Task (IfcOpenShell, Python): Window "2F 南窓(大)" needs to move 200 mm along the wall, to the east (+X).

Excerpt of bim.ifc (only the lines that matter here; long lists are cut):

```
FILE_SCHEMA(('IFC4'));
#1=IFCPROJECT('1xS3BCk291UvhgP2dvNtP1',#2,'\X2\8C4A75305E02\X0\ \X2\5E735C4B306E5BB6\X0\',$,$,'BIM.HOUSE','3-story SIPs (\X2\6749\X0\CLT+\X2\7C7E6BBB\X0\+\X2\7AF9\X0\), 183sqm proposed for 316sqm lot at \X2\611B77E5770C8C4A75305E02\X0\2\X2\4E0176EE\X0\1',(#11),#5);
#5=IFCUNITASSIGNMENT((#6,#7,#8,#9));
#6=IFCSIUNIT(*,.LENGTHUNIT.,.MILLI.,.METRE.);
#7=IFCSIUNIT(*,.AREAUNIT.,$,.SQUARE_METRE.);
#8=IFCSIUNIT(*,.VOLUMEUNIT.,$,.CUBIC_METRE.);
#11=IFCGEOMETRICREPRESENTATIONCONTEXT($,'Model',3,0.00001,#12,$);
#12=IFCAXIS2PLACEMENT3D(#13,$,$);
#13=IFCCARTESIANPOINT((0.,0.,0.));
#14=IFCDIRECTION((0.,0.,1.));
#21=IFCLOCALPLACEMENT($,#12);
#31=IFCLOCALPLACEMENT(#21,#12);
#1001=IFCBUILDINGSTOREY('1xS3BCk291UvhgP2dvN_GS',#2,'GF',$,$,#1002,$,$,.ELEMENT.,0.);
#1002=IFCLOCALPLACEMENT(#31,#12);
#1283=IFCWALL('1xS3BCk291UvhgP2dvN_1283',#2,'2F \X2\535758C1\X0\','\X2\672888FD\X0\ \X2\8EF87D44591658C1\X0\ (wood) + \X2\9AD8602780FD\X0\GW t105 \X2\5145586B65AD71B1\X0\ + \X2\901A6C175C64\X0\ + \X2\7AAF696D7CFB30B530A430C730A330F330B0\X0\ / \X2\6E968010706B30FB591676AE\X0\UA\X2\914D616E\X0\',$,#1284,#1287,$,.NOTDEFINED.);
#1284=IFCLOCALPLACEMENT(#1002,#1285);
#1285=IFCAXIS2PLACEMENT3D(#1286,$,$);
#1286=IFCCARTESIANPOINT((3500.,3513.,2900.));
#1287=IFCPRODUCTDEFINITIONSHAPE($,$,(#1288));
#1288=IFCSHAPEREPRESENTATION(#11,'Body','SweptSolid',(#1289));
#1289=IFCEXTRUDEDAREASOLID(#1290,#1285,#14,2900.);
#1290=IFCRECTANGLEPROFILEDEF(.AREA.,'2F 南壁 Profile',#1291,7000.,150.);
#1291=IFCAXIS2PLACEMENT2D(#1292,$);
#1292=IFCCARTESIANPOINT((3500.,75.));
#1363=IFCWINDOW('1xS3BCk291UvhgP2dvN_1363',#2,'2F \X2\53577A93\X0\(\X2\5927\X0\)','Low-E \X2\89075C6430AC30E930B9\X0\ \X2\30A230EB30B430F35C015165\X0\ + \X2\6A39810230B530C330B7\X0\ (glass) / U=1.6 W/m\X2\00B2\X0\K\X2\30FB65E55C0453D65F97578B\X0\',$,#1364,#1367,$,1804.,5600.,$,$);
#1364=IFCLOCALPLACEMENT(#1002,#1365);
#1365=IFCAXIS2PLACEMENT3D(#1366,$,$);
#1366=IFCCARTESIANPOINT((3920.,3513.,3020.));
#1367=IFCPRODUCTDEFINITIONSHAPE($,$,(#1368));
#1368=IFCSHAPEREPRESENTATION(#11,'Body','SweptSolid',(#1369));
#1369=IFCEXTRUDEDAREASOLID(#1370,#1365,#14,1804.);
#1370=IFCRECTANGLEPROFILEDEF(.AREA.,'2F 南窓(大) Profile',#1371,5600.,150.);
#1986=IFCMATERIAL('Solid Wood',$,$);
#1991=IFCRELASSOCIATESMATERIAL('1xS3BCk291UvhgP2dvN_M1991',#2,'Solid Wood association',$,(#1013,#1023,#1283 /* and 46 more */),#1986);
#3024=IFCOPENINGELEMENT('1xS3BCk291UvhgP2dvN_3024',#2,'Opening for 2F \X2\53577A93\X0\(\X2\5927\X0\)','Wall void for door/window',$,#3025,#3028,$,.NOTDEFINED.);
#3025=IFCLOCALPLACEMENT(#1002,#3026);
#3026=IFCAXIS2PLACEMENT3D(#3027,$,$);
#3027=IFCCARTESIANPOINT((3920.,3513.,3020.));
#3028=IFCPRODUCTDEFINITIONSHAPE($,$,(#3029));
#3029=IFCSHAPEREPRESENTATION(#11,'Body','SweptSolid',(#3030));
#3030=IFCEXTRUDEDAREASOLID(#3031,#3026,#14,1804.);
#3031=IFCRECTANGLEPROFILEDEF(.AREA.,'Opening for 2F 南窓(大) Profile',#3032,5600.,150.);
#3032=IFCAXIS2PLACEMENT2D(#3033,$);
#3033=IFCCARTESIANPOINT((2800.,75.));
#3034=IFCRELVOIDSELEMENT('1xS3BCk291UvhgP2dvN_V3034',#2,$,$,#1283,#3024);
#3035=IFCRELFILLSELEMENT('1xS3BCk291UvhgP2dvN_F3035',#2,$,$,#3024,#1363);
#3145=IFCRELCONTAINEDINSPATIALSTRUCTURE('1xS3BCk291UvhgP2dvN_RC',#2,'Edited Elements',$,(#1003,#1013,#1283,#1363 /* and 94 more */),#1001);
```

```python
import ifcopenshell
import ifcopenshell.api.geometry
import ifcopenshell.util.placement
import ifcopenshell.util.unit

model = ifcopenshell.open("bim.ifc")
unit_scale = ifcopenshell.util.unit.calculate_unit_scale(model)

window = model.by_guid("1xS3BCk291UvhgP2dvN_1363")
opening = window.FillsVoids[0].RelatingOpeningElement
wall = opening.VoidsElements[0].RelatingBuildingElement

wall_matrix = ifcopenshell.util.placement.get_local_placement(wall.ObjectPlacement)
shift = wall_matrix[:3, 0] * 0.2 / unit_scale
before = ifcopenshell.util.placement.get_local_placement(window.ObjectPlacement)[:3, 3].copy()

# The window is not placed relative to its opening, so move both.
for product in (opening, window):
    matrix = ifcopenshell.util.placement.get_local_placement(product.ObjectPlacement)
    matrix[:3, 3] += shift
    ifcopenshell.api.geometry.edit_object_placement(model, product=product, matrix=matrix, is_si=False)

after = ifcopenshell.util.placement.get_local_placement(window.ObjectPlacement)[:3, 3]
print("window moved by", (after - before).round(3) + 0.0)

model.write("bim_rev.ifc")
```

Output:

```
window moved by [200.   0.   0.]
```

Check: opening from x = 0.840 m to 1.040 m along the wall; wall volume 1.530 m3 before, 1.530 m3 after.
